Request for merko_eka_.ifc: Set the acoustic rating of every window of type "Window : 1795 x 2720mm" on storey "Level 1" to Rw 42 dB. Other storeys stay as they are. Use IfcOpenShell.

First a look at what the model holds.

```python
import ifcopenshell
import ifcopenshell.util.element

model = ifcopenshell.open("merko_eka_.ifc")
print(model.schema)
storey = next(s for s in model.by_type("IfcBuildingStorey") if s.Name == "Level 1")
windows = [e for e in ifcopenshell.util.element.get_decomposition(storey) if e.is_a("IfcWindow")]
seen = {}
for e in windows:
    element_type = ifcopenshell.util.element.get_type(e)
    key = (element_type.Name if element_type != e and element_type else None, ifcopenshell.util.element.get_pset(e, "Pset_WindowCommon", "AcousticRating"))
    seen[key] = seen.get(key, 0) + 1
for (name, value), count in sorted(seen.items(), key=str):
    print(count, "x", name, "|", value)
```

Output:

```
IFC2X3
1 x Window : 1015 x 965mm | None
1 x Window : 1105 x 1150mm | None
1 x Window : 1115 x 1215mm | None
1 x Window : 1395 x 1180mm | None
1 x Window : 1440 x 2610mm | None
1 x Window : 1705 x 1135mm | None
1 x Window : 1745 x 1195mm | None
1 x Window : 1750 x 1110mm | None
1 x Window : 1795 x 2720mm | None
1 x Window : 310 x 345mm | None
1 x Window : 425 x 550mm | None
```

```python
import ifcopenshell
import ifcopenshell.api.pset
import ifcopenshell.util.element

model = ifcopenshell.open("merko_eka_.ifc")

storey = next(s for s in model.by_type("IfcBuildingStorey") if s.Name == "Level 1")
windows = [e for e in ifcopenshell.util.element.get_decomposition(storey) if e.is_a("IfcWindow")]

count = 0
for e in windows:
    element_type = ifcopenshell.util.element.get_type(e)
    if element_type in (None, e) or element_type.Name != "Window : 1795 x 2720mm":
        continue
    # add_pset returns the element's existing set when there is one.
    pset = ifcopenshell.api.pset.add_pset(model, product=e, name="Pset_WindowCommon")
    ifcopenshell.api.pset.edit_pset(model, pset=pset, properties={"AcousticRating": "Rw 42 dB"})
    count += 1

print(count, "windows updated")

model.write("merko_eka__rev.ifc")
```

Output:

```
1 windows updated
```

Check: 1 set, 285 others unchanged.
